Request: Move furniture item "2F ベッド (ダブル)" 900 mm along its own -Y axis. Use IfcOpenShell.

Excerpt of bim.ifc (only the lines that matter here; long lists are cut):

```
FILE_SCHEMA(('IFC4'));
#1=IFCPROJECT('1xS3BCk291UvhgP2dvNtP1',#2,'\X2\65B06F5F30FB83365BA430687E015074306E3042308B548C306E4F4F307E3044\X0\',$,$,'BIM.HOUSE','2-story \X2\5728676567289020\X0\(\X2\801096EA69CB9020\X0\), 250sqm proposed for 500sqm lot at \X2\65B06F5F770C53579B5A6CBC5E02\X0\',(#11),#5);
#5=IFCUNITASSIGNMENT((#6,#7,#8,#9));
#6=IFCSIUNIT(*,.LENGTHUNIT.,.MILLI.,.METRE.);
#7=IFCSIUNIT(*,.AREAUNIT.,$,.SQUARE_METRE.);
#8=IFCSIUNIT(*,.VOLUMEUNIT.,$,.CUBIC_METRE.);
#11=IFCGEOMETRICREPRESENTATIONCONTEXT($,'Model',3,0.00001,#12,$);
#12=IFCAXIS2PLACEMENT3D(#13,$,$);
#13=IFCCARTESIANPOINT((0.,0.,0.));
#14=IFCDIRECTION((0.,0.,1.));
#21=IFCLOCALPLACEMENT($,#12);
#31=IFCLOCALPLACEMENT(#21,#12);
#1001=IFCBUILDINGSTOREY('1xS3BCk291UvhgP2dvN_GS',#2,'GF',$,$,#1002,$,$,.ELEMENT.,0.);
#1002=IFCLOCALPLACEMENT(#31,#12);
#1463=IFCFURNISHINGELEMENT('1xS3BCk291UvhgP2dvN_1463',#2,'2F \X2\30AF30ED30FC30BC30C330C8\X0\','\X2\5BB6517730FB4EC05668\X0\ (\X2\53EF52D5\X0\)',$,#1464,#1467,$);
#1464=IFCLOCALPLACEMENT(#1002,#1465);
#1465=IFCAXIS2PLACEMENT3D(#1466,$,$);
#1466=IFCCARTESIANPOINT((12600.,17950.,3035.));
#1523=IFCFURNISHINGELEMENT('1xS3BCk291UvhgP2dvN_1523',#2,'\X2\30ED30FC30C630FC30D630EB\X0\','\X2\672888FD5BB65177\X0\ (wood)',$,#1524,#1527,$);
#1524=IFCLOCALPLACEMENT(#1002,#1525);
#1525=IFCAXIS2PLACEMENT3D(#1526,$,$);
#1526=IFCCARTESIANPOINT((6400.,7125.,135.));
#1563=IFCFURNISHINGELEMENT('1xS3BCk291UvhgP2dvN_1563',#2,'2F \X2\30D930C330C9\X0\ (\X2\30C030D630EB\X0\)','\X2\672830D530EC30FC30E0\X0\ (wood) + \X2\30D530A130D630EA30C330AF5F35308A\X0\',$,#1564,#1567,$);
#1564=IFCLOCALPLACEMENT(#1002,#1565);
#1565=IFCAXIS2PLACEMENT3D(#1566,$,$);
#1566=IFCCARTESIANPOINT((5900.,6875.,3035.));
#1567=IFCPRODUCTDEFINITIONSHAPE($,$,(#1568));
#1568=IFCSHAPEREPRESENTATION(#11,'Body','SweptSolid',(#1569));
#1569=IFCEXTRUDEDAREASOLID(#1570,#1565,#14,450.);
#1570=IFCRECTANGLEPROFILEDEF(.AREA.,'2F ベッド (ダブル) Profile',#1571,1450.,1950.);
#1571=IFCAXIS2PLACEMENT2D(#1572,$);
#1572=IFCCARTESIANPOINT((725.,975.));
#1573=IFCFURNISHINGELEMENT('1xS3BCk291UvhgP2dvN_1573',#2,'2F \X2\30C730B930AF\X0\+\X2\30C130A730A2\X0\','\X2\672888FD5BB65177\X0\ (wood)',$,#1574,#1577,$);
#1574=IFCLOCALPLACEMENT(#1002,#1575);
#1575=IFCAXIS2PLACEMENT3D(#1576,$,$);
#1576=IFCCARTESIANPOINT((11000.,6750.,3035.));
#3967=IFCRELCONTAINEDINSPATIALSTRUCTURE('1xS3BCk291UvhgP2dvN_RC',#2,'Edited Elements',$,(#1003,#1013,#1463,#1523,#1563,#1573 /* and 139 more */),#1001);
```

```python
import ifcopenshell
import ifcopenshell.api.geometry
import ifcopenshell.util.placement
import ifcopenshell.util.unit

model = ifcopenshell.open("bim.ifc")
unit_scale = ifcopenshell.util.unit.calculate_unit_scale(model)

item = model.by_id(1563)
matrix = ifcopenshell.util.placement.get_local_placement(item.ObjectPlacement)
matrix[:3, 3] -= matrix[:3, 1] * 0.9 / unit_scale
ifcopenshell.api.geometry.edit_object_placement(model, product=item, matrix=matrix, is_si=False)

print(ifcopenshell.util.placement.get_local_placement(item.ObjectPlacement).round(3) + 0.0)

model.write("bim-out.ifc")
```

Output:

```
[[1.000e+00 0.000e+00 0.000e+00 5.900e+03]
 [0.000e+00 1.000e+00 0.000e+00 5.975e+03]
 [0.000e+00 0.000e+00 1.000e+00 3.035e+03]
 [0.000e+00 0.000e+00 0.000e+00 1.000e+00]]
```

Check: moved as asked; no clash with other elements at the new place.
